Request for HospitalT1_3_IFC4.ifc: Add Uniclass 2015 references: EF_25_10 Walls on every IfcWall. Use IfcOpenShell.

First a look at what the model holds.

```python
import ifcopenshell

model = ifcopenshell.open("HospitalT1_3_IFC4.ifc")
print(model.schema)
print("classifications:", [c.Name for c in model.by_type("IfcClassification")])
for ifc_class in ("IfcDoor", "IfcRoof", "IfcStair", "IfcWall", "IfcWindow"):
    print(ifc_class, len(model.by_type(ifc_class)))
```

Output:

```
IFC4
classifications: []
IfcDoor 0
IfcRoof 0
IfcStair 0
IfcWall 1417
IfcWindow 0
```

```python
import ifcopenshell
import ifcopenshell.api.classification

model = ifcopenshell.open("HospitalT1_3_IFC4.ifc")

system = ifcopenshell.api.classification.add_classification(model, classification="Uniclass 2015")

codes = {
    "IfcWall": ("EF_25_10", "Walls"),
}
for ifc_class, (code, name) in codes.items():
    products = model.by_type(ifc_class)
    ifcopenshell.api.classification.add_reference(
        model, products=products, classification=system, identification=code, name=name
    )
    print(code, len(products))

model.write("HospitalT1_3_IFC4-out.ifc")
```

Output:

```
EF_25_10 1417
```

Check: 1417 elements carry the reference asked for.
